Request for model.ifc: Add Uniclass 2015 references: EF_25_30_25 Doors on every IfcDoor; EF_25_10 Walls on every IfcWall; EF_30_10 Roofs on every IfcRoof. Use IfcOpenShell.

First a look at what the model holds.

```python
import ifcopenshell

model = ifcopenshell.open("model.ifc")
print(model.schema)
print("classifications:", [c.Name for c in model.by_type("IfcClassification")])
for ifc_class in ("IfcDoor", "IfcRoof", "IfcStair", "IfcWall", "IfcWindow"):
    print(ifc_class, len(model.by_type(ifc_class)))
```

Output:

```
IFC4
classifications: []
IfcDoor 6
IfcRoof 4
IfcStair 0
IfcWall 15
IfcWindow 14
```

```python
import ifcopenshell
import ifcopenshell.api.classification

model = ifcopenshell.open("model.ifc")

system = ifcopenshell.api.classification.add_classification(model, classification="Uniclass 2015")

codes = {
    "IfcDoor": ("EF_25_30_25", "Doors"),
    "IfcWall": ("EF_25_10", "Walls"),
    "IfcRoof": ("EF_30_10", "Roofs"),
}
for ifc_class, (code, name) in codes.items():
    products = model.by_type(ifc_class)
    ifcopenshell.api.classification.add_reference(
        model, products=products, classification=system, identification=code, name=name
    )
    print(code, len(products))

model.write("model_v2.ifc")
```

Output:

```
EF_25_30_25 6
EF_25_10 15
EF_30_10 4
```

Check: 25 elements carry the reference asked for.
